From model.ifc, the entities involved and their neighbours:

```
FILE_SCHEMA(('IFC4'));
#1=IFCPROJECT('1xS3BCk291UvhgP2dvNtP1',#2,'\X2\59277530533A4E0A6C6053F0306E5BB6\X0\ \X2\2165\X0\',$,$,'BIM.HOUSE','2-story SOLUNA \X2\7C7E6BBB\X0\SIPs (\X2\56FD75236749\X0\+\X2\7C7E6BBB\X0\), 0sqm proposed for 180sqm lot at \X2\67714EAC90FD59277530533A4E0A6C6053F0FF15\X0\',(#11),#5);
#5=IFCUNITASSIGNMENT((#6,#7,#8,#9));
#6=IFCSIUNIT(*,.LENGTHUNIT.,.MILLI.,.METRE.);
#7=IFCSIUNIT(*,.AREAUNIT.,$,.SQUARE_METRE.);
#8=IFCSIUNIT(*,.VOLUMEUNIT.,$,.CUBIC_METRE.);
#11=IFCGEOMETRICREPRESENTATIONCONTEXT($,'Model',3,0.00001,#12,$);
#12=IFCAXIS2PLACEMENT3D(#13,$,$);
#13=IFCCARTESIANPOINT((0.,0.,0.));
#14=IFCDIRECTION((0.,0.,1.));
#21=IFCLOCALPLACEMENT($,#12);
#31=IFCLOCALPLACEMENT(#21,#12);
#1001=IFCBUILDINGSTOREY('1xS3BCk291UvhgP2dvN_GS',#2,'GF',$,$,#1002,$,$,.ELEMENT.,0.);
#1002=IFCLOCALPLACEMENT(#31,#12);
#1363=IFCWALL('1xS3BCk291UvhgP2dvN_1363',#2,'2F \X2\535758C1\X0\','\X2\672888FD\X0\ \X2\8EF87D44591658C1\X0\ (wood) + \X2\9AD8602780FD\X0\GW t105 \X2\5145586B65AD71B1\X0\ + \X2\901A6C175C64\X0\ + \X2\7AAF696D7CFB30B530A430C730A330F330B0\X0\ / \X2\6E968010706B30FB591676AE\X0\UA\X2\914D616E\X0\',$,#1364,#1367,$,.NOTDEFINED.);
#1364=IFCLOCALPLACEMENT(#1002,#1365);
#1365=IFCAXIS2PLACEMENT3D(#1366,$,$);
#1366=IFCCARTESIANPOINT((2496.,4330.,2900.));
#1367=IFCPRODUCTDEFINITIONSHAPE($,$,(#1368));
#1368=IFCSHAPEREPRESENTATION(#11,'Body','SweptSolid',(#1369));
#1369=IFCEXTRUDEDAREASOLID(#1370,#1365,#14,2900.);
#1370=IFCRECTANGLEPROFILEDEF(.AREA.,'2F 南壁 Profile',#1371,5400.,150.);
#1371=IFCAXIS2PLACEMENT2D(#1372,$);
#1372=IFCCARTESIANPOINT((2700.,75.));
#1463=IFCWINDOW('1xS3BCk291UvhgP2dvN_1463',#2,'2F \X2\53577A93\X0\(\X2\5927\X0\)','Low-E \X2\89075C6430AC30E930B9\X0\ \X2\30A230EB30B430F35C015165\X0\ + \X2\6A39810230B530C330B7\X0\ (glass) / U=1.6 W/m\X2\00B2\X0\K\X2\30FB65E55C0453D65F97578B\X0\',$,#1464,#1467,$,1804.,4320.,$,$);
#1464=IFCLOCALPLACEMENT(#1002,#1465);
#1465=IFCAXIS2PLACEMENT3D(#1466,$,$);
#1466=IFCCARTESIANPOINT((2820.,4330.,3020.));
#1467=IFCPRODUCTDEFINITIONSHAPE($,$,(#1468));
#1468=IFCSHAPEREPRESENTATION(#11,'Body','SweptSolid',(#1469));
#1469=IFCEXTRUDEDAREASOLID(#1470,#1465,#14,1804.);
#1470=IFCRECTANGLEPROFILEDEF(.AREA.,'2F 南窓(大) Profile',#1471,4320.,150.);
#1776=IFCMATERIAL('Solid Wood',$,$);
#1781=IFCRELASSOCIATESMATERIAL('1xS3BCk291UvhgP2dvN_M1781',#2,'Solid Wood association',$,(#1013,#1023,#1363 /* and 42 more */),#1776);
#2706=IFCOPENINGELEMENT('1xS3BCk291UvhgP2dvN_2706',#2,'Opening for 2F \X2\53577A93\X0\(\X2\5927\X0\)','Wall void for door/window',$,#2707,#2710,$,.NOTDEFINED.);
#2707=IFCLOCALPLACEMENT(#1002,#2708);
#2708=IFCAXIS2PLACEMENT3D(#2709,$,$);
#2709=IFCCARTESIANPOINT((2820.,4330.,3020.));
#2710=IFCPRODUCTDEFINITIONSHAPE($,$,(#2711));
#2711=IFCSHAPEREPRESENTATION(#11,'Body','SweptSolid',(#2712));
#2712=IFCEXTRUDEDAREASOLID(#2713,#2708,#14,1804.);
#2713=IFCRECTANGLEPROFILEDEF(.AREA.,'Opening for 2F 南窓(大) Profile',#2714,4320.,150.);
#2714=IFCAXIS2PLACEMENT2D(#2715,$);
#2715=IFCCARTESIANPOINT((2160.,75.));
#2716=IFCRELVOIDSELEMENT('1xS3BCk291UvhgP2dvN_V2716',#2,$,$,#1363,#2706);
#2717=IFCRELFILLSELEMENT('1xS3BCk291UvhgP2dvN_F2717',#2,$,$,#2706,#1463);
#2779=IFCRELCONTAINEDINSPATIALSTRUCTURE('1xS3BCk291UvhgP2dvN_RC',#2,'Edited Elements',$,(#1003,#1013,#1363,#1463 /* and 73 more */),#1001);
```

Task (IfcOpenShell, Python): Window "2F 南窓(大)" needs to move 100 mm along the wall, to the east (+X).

```python
import ifcopenshell
import ifcopenshell.api.geometry
import ifcopenshell.util.placement
import ifcopenshell.util.unit

model = ifcopenshell.open("model.ifc")
unit_scale = ifcopenshell.util.unit.calculate_unit_scale(model)

window = model.by_id(1463)
opening = window.FillsVoids[0].RelatingOpeningElement
wall = opening.VoidsElements[0].RelatingBuildingElement

wall_matrix = ifcopenshell.util.placement.get_local_placement(wall.ObjectPlacement)
shift = wall_matrix[:3, 0] * 0.1 / unit_scale
before = ifcopenshell.util.placement.get_local_placement(window.ObjectPlacement)[:3, 3].copy()

# The window is not placed relative to its opening, so move both.
for product in (opening, window):
    matrix = ifcopenshell.util.placement.get_local_placement(product.ObjectPlacement)
    matrix[:3, 3] += shift
    ifcopenshell.api.geometry.edit_object_placement(model, product=product, matrix=matrix, is_si=False)

after = ifcopenshell.util.placement.get_local_placement(window.ObjectPlacement)[:3, 3]
print("window moved by", (after - before).round(3) + 0.0)

model.write("model_edited.ifc")
```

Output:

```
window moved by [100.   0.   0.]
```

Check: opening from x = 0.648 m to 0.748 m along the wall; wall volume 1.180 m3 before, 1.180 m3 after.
